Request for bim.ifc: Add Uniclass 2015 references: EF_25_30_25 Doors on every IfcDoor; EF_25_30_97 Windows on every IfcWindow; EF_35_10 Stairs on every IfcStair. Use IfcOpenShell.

First a look at what the model holds.

```python
import ifcopenshell

model = ifcopenshell.open("bim.ifc")
print(model.schema)
print("classifications:", [c.Name for c in model.by_type("IfcClassification")])
for ifc_class in ("IfcDoor", "IfcRoof", "IfcStair", "IfcWall", "IfcWindow"):
    print(ifc_class, len(model.by_type(ifc_class)))
```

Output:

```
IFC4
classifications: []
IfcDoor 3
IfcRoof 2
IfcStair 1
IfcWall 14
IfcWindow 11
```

```python
import ifcopenshell
import ifcopenshell.api.classification

model = ifcopenshell.open("bim.ifc")

system = ifcopenshell.api.classification.add_classification(model, classification="Uniclass 2015")

codes = {
    "IfcDoor": ("EF_25_30_25", "Doors"),
    "IfcWindow": ("EF_25_30_97", "Windows"),
    "IfcStair": ("EF_35_10", "Stairs"),
}
for ifc_class, (code, name) in codes.items():
    products = model.by_type(ifc_class)
    ifcopenshell.api.classification.add_reference(
        model, products=products, classification=system, identification=code, name=name
    )
    print(code, len(products))

model.write("bim_v2.ifc")
```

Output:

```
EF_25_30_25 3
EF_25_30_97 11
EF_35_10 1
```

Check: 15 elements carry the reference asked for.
